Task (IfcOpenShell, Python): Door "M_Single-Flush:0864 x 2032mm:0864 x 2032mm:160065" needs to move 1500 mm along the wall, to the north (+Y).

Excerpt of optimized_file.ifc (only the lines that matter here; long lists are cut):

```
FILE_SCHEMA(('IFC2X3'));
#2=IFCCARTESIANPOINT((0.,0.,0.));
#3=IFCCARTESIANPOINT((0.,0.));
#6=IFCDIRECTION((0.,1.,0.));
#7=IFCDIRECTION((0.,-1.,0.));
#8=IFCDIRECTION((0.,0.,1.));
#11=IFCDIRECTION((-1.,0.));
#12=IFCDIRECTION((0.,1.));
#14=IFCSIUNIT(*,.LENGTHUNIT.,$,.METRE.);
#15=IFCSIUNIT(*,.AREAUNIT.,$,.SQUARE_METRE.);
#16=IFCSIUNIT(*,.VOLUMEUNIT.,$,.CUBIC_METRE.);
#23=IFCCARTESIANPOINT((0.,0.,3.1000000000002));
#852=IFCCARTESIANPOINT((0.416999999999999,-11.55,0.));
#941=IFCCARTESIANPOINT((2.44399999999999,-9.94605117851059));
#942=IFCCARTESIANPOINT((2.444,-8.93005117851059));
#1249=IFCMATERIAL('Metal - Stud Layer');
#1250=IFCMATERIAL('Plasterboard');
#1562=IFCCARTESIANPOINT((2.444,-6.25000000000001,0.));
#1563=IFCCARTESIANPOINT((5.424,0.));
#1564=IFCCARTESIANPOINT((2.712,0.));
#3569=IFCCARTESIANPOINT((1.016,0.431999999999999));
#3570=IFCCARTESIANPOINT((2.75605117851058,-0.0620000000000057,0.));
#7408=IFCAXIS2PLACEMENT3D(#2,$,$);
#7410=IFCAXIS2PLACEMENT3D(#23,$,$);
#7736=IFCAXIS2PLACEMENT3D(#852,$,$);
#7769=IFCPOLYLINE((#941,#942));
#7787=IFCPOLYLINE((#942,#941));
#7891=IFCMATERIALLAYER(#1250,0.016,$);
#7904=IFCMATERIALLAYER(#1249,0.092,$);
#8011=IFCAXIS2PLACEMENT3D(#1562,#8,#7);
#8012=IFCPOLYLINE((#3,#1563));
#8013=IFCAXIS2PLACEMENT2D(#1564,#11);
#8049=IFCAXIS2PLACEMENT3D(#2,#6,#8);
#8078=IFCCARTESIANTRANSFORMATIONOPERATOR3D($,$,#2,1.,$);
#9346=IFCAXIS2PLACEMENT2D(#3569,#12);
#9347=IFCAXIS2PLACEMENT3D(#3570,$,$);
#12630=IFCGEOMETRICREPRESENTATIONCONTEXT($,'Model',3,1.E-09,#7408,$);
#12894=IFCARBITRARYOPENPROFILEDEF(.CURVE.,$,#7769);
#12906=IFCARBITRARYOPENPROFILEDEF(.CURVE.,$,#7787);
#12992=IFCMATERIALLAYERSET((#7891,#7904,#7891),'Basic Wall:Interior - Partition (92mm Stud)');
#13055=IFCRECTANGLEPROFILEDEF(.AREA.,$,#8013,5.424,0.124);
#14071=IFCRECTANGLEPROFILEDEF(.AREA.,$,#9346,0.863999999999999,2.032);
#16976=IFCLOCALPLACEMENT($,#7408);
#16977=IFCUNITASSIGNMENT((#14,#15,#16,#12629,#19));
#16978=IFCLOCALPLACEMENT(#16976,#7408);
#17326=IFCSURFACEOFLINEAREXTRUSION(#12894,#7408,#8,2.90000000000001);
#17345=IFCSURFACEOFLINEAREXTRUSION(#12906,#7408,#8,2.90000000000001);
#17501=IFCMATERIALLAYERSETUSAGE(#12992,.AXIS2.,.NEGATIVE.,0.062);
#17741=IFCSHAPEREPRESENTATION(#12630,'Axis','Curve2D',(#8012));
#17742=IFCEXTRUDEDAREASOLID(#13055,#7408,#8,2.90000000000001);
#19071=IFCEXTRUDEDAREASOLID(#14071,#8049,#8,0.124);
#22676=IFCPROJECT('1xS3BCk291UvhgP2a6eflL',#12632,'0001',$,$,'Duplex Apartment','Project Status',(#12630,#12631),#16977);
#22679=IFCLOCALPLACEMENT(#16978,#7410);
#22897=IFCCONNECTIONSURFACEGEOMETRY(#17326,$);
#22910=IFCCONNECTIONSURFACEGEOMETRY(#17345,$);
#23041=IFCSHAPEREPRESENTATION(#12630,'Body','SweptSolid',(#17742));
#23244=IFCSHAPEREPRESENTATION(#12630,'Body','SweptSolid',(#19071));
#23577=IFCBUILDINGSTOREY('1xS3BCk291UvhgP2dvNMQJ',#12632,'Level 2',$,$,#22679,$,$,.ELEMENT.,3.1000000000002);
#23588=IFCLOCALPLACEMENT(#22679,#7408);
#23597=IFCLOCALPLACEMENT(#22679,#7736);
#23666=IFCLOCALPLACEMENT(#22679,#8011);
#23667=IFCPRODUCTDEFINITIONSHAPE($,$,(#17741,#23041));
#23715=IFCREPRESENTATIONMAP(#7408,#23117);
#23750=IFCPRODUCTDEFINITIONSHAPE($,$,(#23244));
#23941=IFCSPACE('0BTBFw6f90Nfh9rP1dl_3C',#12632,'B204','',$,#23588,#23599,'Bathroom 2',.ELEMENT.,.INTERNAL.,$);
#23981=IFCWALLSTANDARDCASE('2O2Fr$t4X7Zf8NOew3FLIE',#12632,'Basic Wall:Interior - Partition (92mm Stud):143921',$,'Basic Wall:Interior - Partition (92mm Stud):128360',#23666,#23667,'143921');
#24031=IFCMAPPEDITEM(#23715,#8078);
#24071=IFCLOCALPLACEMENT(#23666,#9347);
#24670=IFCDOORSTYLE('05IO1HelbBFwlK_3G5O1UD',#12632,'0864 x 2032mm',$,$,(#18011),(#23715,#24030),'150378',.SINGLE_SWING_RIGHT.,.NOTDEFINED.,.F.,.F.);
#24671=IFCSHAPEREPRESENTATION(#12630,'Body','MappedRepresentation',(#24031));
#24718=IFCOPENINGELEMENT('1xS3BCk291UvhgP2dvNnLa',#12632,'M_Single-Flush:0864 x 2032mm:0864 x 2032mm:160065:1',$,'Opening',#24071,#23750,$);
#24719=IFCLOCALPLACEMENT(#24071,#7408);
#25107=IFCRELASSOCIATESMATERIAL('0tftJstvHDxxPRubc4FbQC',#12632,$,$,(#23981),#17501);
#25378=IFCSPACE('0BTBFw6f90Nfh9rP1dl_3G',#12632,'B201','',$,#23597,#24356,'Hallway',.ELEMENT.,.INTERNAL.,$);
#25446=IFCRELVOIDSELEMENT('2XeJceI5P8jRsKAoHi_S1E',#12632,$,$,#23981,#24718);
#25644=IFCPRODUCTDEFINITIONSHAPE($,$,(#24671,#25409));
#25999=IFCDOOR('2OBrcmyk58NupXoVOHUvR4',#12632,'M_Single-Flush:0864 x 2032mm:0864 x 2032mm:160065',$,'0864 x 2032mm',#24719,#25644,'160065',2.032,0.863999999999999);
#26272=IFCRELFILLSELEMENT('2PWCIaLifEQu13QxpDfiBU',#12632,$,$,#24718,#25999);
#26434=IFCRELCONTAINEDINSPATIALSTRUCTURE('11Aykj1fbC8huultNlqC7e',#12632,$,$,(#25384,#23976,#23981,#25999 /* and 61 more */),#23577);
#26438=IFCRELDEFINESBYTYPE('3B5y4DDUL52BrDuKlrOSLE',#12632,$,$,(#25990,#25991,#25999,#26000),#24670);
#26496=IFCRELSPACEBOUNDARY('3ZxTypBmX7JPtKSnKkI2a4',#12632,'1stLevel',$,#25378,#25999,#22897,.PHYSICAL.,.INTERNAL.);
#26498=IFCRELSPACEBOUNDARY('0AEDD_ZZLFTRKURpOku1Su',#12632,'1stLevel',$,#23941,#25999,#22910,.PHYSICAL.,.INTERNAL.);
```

```python
import numpy as np
import ifcopenshell
import ifcopenshell.api.geometry
import ifcopenshell.util.placement

model = ifcopenshell.open("optimized_file.ifc")

door = model.by_guid("2OBrcmyk58NupXoVOHUvR4")
opening = door.FillsVoids[0].RelatingOpeningElement
wall = opening.VoidsElements[0].RelatingBuildingElement

wall_matrix = ifcopenshell.util.placement.get_local_placement(wall.ObjectPlacement)
shift = wall_matrix[:3, 0] * -1.5
before = ifcopenshell.util.placement.get_local_placement(door.ObjectPlacement)[:3, 3].copy()

# The door is placed relative to its opening, so it follows when the opening moves.
matrix = ifcopenshell.util.placement.get_local_placement(opening.ObjectPlacement)
matrix[:3, 3] += shift
ifcopenshell.api.geometry.edit_object_placement(
    model, product=opening, matrix=matrix, is_si=False, should_transform_children=True
)

# Space boundary surfaces are stored in each space's coordinates; move them too.
for rel in door.ProvidesBoundaries:
    if not rel.ConnectionGeometry:
        continue
    surface = rel.ConnectionGeometry.SurfaceOnRelatingElement
    space_matrix = ifcopenshell.util.placement.get_local_placement(rel.RelatingSpace.ObjectPlacement)
    point = np.array(surface.Position.Location.Coordinates) + space_matrix[:3, :3].T @ shift
    surface.Position = model.createIfcAxis2Placement3D(
        model.createIfcCartesianPoint(point.tolist()), surface.Position.Axis, surface.Position.RefDirection
    )

after = ifcopenshell.util.placement.get_local_placement(door.ObjectPlacement)[:3, 3]
print("door moved by", (after - before).round(3) + 0.0)

model.write("optimized_file_v2.ifc")
```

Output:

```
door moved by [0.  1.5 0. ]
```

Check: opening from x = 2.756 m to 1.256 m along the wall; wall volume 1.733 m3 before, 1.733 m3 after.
